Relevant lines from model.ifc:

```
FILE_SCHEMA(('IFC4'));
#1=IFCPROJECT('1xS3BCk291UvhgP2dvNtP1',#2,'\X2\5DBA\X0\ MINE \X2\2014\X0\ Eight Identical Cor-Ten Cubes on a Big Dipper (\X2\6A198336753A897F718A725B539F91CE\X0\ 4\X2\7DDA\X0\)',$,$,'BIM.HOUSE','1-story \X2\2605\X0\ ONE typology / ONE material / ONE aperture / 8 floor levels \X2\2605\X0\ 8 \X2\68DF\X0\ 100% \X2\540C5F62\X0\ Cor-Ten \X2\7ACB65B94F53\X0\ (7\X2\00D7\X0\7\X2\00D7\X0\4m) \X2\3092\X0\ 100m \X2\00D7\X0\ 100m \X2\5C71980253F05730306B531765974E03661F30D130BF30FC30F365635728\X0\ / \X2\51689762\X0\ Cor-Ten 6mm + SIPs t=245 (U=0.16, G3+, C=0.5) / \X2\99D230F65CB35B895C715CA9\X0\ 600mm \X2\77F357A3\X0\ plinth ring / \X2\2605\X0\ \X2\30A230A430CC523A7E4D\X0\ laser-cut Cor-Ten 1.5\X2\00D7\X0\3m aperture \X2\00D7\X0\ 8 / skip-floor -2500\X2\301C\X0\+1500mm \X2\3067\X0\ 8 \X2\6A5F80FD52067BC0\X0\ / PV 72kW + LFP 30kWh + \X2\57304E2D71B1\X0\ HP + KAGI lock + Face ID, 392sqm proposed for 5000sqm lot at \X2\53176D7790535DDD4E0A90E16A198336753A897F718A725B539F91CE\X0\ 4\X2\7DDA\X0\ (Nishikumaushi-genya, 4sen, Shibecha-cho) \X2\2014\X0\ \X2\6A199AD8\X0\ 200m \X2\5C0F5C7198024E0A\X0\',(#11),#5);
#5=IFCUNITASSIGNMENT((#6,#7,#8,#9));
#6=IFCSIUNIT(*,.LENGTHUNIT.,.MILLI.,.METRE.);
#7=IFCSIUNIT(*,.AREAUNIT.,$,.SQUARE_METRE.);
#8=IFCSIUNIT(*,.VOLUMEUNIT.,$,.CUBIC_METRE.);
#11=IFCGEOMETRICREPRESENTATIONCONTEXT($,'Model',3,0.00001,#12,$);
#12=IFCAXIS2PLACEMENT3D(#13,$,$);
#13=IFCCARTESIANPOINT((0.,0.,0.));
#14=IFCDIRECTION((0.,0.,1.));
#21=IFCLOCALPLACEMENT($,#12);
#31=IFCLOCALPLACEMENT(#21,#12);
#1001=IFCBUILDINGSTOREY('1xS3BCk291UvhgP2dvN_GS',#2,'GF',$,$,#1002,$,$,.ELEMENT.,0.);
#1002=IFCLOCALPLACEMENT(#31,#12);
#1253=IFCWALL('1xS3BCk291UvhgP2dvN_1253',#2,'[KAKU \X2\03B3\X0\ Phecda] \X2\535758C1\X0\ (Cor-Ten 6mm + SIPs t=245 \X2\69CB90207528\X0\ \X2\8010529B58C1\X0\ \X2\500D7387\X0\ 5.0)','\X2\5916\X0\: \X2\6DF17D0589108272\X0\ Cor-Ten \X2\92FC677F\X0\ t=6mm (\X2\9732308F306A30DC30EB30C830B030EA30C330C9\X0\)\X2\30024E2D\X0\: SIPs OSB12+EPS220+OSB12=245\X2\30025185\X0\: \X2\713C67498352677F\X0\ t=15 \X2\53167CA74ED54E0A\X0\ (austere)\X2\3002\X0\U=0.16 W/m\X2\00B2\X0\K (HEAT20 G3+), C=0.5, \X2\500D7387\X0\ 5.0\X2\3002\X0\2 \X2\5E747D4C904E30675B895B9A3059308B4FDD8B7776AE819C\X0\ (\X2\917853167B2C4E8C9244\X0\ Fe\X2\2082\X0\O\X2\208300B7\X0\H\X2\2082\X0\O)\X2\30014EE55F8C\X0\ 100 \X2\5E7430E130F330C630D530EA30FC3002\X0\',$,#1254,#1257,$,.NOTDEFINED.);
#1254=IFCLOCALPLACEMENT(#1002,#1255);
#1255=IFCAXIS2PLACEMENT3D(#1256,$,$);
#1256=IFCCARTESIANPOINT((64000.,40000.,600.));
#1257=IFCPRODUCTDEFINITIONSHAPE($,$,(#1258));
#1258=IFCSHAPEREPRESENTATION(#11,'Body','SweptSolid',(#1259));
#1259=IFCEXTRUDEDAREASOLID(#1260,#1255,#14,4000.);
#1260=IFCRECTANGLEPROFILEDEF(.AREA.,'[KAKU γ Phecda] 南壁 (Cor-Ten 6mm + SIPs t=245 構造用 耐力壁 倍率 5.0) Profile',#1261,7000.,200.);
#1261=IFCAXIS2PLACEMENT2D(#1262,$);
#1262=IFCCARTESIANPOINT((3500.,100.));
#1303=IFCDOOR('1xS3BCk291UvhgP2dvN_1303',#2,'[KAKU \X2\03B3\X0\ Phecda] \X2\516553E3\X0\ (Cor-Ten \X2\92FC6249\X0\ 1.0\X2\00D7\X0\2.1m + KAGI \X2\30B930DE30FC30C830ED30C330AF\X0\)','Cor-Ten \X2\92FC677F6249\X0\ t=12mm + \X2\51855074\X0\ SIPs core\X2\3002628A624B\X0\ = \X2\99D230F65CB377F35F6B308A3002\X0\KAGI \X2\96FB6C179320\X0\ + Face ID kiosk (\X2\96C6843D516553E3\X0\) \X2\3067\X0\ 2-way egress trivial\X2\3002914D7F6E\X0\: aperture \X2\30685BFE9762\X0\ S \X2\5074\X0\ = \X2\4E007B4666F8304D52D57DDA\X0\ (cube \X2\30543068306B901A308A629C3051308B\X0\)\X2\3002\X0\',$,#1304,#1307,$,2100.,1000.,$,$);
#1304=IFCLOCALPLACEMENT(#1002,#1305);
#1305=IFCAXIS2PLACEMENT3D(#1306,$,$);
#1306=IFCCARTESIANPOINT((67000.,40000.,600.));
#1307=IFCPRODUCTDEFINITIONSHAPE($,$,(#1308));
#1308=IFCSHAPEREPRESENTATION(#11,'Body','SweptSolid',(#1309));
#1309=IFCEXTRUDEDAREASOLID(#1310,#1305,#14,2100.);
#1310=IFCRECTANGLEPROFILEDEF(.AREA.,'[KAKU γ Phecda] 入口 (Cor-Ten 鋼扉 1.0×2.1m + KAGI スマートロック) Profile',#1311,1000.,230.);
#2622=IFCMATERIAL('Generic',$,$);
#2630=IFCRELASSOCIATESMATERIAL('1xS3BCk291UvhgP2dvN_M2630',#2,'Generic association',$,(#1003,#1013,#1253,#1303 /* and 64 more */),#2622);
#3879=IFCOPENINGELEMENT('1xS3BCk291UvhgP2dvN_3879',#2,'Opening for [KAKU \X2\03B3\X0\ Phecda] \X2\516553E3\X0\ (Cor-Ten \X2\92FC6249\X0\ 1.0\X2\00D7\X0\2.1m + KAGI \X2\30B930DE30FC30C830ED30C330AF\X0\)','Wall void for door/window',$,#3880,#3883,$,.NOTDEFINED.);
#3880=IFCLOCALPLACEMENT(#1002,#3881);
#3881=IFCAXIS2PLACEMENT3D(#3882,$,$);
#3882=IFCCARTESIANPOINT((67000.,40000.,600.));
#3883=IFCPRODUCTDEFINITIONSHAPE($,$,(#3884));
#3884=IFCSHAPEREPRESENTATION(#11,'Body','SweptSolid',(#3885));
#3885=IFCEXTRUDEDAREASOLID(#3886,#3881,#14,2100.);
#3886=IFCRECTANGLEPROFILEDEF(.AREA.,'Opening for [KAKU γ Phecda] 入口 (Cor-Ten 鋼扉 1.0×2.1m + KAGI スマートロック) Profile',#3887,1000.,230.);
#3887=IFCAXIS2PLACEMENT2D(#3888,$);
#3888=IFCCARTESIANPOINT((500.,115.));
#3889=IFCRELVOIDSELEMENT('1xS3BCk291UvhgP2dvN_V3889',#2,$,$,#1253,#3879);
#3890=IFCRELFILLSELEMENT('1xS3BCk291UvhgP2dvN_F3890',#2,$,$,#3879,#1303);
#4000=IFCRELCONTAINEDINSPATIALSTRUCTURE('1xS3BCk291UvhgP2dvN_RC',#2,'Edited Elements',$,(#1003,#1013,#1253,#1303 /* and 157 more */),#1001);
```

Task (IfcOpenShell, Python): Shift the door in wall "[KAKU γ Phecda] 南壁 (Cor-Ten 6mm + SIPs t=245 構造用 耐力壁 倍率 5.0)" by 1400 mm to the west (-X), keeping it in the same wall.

```python
import ifcopenshell
import ifcopenshell.api.geometry
import ifcopenshell.util.placement

model = ifcopenshell.open("model.ifc")

door = model.by_guid("1xS3BCk291UvhgP2dvN_1303")
opening = door.FillsVoids[0].RelatingOpeningElement
wall = opening.VoidsElements[0].RelatingBuildingElement

wall_matrix = ifcopenshell.util.placement.get_local_placement(wall.ObjectPlacement)
shift = wall_matrix[:3, 0] * -1400.0
before = ifcopenshell.util.placement.get_local_placement(door.ObjectPlacement)[:3, 3].copy()

# The door is not placed relative to its opening, so move both.
for product in (opening, door):
    matrix = ifcopenshell.util.placement.get_local_placement(product.ObjectPlacement)
    matrix[:3, 3] += shift
    ifcopenshell.api.geometry.edit_object_placement(model, product=product, matrix=matrix, is_si=False)

after = ifcopenshell.util.placement.get_local_placement(door.ObjectPlacement)[:3, 3]
print("door moved by", (after - before).round(3) + 0.0)

model.write("model_edited.ifc")
```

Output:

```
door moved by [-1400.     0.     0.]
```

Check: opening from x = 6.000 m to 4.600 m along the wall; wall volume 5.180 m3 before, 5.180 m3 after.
